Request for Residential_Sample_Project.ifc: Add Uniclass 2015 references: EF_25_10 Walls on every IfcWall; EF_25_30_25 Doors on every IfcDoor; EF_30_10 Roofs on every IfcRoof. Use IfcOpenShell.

First a look at what the model holds.

```python
import ifcopenshell

model = ifcopenshell.open("Residential_Sample_Project.ifc")
print(model.schema)
print("classifications:", [c.Name for c in model.by_type("IfcClassification")])
for ifc_class in ("IfcDoor", "IfcRoof", "IfcStair", "IfcWall", "IfcWindow"):
    print(ifc_class, len(model.by_type(ifc_class)))
```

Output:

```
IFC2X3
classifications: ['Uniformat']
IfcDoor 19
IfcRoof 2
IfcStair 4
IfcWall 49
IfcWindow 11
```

```python
import ifcopenshell
import ifcopenshell.api.classification

model = ifcopenshell.open("Residential_Sample_Project.ifc")

# IFC2X3 requires Source and Edition and has no link from the project to the system.
system = model.create_entity("IfcClassification", Source="NBS", Edition="2015", Name="Uniclass 2015")

codes = {
    "IfcWall": ("EF_25_10", "Walls"),
    "IfcDoor": ("EF_25_30_25", "Doors"),
    "IfcRoof": ("EF_30_10", "Roofs"),
}
for ifc_class, (code, name) in codes.items():
    products = model.by_type(ifc_class)
    ifcopenshell.api.classification.add_reference(
        model, products=products, classification=system, identification=code, name=name
    )
    print(code, len(products))

model.write("Residential_Sample_Project_v2.ifc")
```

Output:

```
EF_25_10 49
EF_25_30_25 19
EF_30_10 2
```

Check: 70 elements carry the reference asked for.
